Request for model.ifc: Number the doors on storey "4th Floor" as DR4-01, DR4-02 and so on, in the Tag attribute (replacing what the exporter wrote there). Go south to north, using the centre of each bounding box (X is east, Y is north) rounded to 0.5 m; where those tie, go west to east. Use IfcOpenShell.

First a look at what the model holds.

```python
import ifcopenshell
import ifcopenshell.util.element
import ifcopenshell.util.placement

model = ifcopenshell.open("model.ifc")
print(model.schema)
storey = next(s for s in model.by_type("IfcBuildingStorey") if s.Name == "4th Floor")
doors = [e for e in ifcopenshell.util.element.get_decomposition(storey) if e.is_a("IfcDoor")]
for e in sorted(doors, key=lambda e: e.id()):
    origin = ifcopenshell.util.placement.get_local_placement(e.ObjectPlacement)[:3, 3]
    print(e.id(), e.Tag, e.Name, origin.round(2) + 0.0, sep=" | ")
```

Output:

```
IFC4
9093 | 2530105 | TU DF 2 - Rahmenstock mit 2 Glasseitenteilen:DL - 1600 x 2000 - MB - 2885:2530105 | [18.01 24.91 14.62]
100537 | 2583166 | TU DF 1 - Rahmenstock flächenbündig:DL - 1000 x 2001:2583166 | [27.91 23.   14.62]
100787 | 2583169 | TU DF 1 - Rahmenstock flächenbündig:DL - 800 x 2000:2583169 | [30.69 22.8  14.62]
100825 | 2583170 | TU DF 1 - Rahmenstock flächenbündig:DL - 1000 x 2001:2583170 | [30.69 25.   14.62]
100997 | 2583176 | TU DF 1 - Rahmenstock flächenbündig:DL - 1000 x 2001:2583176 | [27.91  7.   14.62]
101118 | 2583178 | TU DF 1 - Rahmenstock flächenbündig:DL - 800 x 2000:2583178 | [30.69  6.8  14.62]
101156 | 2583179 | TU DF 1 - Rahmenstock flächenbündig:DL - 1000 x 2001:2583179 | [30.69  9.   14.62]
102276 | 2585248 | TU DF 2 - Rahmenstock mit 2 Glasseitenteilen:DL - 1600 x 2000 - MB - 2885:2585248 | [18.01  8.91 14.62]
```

```python
import ifcopenshell
import ifcopenshell.geom
import ifcopenshell.util.element
import ifcopenshell.util.shape

model = ifcopenshell.open("model.ifc")
settings = ifcopenshell.geom.settings()
settings.set("use-world-coords", True)


def centre(element):
    shape = ifcopenshell.geom.create_shape(settings, element)
    return ifcopenshell.util.shape.get_bbox_centroid(shape.geometry)


storey = next(s for s in model.by_type("IfcBuildingStorey") if s.Name == "4th Floor")
doors = [e for e in ifcopenshell.util.element.get_decomposition(storey) if e.is_a("IfcDoor")]

# Insertion points can sit at a corner or the storey origin, so sort by the geometry (in metres).
centres = {e: centre(e) for e in doors}
doors.sort(key=lambda e: (round(centres[e][1] / 0.5), centres[e][0]))

for i, e in enumerate(doors, start=1):
    number = f"DR4-{i:02d}"
    e.Tag = number
    print(e.id(), number)

model.write("model_edited.ifc")
```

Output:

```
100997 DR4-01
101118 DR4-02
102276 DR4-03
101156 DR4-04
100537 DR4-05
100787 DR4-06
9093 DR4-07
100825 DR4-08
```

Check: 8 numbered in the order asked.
